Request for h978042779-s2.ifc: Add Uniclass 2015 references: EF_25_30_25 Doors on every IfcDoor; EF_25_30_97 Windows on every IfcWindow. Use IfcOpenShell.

First a look at what the model holds.

```python
import ifcopenshell

model = ifcopenshell.open("h978042779-s2.ifc")
print(model.schema)
print("classifications:", [c.Name for c in model.by_type("IfcClassification")])
for ifc_class in ("IfcDoor", "IfcRoof", "IfcStair", "IfcWall", "IfcWindow"):
    print(ifc_class, len(model.by_type(ifc_class)))
```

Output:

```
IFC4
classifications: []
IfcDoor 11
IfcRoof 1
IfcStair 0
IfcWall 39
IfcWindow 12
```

```python
import ifcopenshell
import ifcopenshell.api.classification

model = ifcopenshell.open("h978042779-s2.ifc")

system = ifcopenshell.api.classification.add_classification(model, classification="Uniclass 2015")

codes = {
    "IfcDoor": ("EF_25_30_25", "Doors"),
    "IfcWindow": ("EF_25_30_97", "Windows"),
}
for ifc_class, (code, name) in codes.items():
    products = model.by_type(ifc_class)
    ifcopenshell.api.classification.add_reference(
        model, products=products, classification=system, identification=code, name=name
    )
    print(code, len(products))

model.write("h978042779-s2_edited.ifc")
```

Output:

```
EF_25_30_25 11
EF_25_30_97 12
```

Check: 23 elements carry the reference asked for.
